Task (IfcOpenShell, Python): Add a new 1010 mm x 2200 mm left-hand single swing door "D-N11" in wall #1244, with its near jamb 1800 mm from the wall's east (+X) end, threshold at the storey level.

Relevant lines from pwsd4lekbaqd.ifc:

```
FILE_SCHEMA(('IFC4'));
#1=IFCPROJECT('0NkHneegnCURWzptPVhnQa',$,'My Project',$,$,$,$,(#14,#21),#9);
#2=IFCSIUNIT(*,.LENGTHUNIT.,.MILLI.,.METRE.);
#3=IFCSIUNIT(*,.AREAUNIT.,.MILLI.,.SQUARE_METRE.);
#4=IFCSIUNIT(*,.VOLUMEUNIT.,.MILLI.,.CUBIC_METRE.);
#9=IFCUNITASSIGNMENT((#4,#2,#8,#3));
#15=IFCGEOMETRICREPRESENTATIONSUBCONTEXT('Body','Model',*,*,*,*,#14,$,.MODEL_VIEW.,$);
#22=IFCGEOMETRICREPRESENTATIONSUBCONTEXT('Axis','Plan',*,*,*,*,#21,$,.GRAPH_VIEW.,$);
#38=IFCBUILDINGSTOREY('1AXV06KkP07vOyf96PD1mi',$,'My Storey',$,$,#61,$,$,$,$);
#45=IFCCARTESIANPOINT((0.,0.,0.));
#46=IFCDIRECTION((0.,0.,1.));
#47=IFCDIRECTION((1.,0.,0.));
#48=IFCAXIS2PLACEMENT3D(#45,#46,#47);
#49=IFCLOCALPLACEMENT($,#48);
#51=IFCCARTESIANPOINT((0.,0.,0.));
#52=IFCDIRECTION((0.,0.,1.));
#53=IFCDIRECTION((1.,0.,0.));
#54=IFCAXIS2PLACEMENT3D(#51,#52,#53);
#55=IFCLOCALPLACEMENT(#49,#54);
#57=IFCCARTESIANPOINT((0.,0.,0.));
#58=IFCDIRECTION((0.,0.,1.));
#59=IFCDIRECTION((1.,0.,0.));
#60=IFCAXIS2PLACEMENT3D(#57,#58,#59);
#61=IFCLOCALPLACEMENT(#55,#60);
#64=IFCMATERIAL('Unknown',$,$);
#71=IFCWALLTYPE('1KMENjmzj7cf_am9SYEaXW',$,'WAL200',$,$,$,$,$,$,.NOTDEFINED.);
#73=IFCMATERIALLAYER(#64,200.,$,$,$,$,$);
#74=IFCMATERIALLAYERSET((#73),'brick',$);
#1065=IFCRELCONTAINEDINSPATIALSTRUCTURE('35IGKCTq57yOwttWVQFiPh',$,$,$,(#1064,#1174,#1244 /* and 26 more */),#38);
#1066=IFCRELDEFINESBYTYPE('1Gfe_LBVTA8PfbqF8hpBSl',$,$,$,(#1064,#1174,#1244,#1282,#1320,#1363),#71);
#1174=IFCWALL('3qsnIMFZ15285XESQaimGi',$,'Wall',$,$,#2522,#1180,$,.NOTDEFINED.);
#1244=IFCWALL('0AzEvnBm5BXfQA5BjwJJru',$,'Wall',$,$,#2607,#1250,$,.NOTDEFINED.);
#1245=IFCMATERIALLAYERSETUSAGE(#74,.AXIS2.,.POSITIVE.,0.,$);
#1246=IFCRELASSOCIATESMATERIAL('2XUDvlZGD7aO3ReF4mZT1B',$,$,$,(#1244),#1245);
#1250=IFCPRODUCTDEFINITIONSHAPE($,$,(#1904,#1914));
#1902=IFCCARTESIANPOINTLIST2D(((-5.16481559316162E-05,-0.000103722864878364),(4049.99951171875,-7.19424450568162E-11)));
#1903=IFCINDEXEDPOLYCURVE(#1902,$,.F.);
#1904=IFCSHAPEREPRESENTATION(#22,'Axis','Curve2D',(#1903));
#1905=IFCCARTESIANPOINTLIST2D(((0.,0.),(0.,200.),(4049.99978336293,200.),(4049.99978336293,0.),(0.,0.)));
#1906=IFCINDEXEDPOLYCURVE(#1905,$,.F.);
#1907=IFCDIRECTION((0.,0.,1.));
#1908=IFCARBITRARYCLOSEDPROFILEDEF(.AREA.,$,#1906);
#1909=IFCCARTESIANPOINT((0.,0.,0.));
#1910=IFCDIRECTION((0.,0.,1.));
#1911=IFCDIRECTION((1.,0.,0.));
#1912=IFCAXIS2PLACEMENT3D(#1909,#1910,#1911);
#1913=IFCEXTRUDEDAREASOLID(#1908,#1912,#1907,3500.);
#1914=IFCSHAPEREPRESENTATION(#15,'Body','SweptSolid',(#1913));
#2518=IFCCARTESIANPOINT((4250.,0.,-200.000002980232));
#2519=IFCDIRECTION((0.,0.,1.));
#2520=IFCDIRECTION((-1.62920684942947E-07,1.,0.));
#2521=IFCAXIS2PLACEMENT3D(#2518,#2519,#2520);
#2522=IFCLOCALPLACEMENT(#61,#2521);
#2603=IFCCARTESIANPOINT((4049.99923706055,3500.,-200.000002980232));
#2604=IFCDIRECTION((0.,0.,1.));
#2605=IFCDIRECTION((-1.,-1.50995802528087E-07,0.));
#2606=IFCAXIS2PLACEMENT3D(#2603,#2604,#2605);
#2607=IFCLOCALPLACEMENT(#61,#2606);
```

```python
import numpy as np
import ifcopenshell
import ifcopenshell.api.feature
import ifcopenshell.api.geometry
import ifcopenshell.api.root
import ifcopenshell.api.spatial
import ifcopenshell.geom
import ifcopenshell.util.element
import ifcopenshell.util.placement
import ifcopenshell.util.representation
import ifcopenshell.util.shape
import ifcopenshell.util.unit

model = ifcopenshell.open("pwsd4lekbaqd.ifc")
unit_scale = ifcopenshell.util.unit.calculate_unit_scale(model)
settings = ifcopenshell.geom.settings()


def volume(element):
    """Net volume in cubic metres, openings subtracted."""
    shape = ifcopenshell.geom.create_shape(settings, element)
    return ifcopenshell.util.shape.get_volume(shape.geometry)


wall = model.by_id(1244)
storey = ifcopenshell.util.element.get_container(wall, ifc_class="IfcBuildingStorey")
context = ifcopenshell.util.representation.get_context(model, "Model", "Body", "MODEL_VIEW")
before = volume(wall)

width, height, from_end, sill = 1.01, 2.2, 1.8, 0.0  # metres

# The wall runs along its own X axis, and the end named is its -X end.
wall_shape = ifcopenshell.geom.create_shape(settings, wall)
x, y, z = ifcopenshell.util.shape.get_vertices(wall_shape.geometry).T
start = x.min() + from_end
face, thickness = float(y.min()), float(y.max() - y.min())
wall_matrix = ifcopenshell.util.placement.get_local_placement(wall.ObjectPlacement)
level = ifcopenshell.util.placement.get_local_placement(storey.ObjectPlacement)[2, 3]


def in_wall(x, y):
    """Placement at x, y metres in the wall's axes, at sill height."""
    matrix = wall_matrix.copy()
    matrix[:, 3] = wall_matrix @ np.array([x / unit_scale, y / unit_scale, 0.0, 1.0])
    matrix[2, 3] = level + sill / unit_scale
    return matrix


# Opening: a box that overshoots both wall faces by 50 mm.
opening = ifcopenshell.api.root.create_entity(model, ifc_class="IfcOpeningElement", predefined_type="OPENING")
box = ifcopenshell.api.geometry.add_wall_representation(
    model, context=context, length=width, height=height, thickness=thickness + 0.1
)
ifcopenshell.api.geometry.assign_representation(model, product=opening, representation=box)
ifcopenshell.api.geometry.edit_object_placement(model, product=opening, matrix=in_wall(start, face - 0.05), is_si=False)
ifcopenshell.api.feature.add_feature(model, feature=opening, element=wall)

door = ifcopenshell.api.root.create_entity(model, ifc_class="IfcDoor", name="D-N11", predefined_type="DOOR")
door.OverallWidth, door.OverallHeight = width / unit_scale, height / unit_scale
door.OperationType = "SINGLE_SWING_LEFT"
body = ifcopenshell.api.geometry.add_door_representation(
    model,
    context=context,
    overall_width=door.OverallWidth,
    overall_height=door.OverallHeight,
    operation_type="SINGLE_SWING_LEFT",
    lining_properties={"LiningDepth": thickness / unit_scale, "ThresholdDepth": thickness / unit_scale},
)
ifcopenshell.api.geometry.assign_representation(model, product=door, representation=body)
ifcopenshell.api.spatial.assign_container(model, products=[door], relating_structure=storey)
ifcopenshell.api.feature.add_filling(model, opening=opening, element=door)

# The lining spans the wall, so the door starts at the wall face.
ifcopenshell.api.geometry.edit_object_placement(model, product=door, matrix=in_wall(start, face), is_si=False)

after = volume(wall)

print(f"wall volume {before:.3f} -> {after:.3f} m3")

model.write("pwsd4lekbaqd_v2.ifc")
```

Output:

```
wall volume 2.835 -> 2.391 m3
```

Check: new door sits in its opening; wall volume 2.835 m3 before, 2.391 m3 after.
